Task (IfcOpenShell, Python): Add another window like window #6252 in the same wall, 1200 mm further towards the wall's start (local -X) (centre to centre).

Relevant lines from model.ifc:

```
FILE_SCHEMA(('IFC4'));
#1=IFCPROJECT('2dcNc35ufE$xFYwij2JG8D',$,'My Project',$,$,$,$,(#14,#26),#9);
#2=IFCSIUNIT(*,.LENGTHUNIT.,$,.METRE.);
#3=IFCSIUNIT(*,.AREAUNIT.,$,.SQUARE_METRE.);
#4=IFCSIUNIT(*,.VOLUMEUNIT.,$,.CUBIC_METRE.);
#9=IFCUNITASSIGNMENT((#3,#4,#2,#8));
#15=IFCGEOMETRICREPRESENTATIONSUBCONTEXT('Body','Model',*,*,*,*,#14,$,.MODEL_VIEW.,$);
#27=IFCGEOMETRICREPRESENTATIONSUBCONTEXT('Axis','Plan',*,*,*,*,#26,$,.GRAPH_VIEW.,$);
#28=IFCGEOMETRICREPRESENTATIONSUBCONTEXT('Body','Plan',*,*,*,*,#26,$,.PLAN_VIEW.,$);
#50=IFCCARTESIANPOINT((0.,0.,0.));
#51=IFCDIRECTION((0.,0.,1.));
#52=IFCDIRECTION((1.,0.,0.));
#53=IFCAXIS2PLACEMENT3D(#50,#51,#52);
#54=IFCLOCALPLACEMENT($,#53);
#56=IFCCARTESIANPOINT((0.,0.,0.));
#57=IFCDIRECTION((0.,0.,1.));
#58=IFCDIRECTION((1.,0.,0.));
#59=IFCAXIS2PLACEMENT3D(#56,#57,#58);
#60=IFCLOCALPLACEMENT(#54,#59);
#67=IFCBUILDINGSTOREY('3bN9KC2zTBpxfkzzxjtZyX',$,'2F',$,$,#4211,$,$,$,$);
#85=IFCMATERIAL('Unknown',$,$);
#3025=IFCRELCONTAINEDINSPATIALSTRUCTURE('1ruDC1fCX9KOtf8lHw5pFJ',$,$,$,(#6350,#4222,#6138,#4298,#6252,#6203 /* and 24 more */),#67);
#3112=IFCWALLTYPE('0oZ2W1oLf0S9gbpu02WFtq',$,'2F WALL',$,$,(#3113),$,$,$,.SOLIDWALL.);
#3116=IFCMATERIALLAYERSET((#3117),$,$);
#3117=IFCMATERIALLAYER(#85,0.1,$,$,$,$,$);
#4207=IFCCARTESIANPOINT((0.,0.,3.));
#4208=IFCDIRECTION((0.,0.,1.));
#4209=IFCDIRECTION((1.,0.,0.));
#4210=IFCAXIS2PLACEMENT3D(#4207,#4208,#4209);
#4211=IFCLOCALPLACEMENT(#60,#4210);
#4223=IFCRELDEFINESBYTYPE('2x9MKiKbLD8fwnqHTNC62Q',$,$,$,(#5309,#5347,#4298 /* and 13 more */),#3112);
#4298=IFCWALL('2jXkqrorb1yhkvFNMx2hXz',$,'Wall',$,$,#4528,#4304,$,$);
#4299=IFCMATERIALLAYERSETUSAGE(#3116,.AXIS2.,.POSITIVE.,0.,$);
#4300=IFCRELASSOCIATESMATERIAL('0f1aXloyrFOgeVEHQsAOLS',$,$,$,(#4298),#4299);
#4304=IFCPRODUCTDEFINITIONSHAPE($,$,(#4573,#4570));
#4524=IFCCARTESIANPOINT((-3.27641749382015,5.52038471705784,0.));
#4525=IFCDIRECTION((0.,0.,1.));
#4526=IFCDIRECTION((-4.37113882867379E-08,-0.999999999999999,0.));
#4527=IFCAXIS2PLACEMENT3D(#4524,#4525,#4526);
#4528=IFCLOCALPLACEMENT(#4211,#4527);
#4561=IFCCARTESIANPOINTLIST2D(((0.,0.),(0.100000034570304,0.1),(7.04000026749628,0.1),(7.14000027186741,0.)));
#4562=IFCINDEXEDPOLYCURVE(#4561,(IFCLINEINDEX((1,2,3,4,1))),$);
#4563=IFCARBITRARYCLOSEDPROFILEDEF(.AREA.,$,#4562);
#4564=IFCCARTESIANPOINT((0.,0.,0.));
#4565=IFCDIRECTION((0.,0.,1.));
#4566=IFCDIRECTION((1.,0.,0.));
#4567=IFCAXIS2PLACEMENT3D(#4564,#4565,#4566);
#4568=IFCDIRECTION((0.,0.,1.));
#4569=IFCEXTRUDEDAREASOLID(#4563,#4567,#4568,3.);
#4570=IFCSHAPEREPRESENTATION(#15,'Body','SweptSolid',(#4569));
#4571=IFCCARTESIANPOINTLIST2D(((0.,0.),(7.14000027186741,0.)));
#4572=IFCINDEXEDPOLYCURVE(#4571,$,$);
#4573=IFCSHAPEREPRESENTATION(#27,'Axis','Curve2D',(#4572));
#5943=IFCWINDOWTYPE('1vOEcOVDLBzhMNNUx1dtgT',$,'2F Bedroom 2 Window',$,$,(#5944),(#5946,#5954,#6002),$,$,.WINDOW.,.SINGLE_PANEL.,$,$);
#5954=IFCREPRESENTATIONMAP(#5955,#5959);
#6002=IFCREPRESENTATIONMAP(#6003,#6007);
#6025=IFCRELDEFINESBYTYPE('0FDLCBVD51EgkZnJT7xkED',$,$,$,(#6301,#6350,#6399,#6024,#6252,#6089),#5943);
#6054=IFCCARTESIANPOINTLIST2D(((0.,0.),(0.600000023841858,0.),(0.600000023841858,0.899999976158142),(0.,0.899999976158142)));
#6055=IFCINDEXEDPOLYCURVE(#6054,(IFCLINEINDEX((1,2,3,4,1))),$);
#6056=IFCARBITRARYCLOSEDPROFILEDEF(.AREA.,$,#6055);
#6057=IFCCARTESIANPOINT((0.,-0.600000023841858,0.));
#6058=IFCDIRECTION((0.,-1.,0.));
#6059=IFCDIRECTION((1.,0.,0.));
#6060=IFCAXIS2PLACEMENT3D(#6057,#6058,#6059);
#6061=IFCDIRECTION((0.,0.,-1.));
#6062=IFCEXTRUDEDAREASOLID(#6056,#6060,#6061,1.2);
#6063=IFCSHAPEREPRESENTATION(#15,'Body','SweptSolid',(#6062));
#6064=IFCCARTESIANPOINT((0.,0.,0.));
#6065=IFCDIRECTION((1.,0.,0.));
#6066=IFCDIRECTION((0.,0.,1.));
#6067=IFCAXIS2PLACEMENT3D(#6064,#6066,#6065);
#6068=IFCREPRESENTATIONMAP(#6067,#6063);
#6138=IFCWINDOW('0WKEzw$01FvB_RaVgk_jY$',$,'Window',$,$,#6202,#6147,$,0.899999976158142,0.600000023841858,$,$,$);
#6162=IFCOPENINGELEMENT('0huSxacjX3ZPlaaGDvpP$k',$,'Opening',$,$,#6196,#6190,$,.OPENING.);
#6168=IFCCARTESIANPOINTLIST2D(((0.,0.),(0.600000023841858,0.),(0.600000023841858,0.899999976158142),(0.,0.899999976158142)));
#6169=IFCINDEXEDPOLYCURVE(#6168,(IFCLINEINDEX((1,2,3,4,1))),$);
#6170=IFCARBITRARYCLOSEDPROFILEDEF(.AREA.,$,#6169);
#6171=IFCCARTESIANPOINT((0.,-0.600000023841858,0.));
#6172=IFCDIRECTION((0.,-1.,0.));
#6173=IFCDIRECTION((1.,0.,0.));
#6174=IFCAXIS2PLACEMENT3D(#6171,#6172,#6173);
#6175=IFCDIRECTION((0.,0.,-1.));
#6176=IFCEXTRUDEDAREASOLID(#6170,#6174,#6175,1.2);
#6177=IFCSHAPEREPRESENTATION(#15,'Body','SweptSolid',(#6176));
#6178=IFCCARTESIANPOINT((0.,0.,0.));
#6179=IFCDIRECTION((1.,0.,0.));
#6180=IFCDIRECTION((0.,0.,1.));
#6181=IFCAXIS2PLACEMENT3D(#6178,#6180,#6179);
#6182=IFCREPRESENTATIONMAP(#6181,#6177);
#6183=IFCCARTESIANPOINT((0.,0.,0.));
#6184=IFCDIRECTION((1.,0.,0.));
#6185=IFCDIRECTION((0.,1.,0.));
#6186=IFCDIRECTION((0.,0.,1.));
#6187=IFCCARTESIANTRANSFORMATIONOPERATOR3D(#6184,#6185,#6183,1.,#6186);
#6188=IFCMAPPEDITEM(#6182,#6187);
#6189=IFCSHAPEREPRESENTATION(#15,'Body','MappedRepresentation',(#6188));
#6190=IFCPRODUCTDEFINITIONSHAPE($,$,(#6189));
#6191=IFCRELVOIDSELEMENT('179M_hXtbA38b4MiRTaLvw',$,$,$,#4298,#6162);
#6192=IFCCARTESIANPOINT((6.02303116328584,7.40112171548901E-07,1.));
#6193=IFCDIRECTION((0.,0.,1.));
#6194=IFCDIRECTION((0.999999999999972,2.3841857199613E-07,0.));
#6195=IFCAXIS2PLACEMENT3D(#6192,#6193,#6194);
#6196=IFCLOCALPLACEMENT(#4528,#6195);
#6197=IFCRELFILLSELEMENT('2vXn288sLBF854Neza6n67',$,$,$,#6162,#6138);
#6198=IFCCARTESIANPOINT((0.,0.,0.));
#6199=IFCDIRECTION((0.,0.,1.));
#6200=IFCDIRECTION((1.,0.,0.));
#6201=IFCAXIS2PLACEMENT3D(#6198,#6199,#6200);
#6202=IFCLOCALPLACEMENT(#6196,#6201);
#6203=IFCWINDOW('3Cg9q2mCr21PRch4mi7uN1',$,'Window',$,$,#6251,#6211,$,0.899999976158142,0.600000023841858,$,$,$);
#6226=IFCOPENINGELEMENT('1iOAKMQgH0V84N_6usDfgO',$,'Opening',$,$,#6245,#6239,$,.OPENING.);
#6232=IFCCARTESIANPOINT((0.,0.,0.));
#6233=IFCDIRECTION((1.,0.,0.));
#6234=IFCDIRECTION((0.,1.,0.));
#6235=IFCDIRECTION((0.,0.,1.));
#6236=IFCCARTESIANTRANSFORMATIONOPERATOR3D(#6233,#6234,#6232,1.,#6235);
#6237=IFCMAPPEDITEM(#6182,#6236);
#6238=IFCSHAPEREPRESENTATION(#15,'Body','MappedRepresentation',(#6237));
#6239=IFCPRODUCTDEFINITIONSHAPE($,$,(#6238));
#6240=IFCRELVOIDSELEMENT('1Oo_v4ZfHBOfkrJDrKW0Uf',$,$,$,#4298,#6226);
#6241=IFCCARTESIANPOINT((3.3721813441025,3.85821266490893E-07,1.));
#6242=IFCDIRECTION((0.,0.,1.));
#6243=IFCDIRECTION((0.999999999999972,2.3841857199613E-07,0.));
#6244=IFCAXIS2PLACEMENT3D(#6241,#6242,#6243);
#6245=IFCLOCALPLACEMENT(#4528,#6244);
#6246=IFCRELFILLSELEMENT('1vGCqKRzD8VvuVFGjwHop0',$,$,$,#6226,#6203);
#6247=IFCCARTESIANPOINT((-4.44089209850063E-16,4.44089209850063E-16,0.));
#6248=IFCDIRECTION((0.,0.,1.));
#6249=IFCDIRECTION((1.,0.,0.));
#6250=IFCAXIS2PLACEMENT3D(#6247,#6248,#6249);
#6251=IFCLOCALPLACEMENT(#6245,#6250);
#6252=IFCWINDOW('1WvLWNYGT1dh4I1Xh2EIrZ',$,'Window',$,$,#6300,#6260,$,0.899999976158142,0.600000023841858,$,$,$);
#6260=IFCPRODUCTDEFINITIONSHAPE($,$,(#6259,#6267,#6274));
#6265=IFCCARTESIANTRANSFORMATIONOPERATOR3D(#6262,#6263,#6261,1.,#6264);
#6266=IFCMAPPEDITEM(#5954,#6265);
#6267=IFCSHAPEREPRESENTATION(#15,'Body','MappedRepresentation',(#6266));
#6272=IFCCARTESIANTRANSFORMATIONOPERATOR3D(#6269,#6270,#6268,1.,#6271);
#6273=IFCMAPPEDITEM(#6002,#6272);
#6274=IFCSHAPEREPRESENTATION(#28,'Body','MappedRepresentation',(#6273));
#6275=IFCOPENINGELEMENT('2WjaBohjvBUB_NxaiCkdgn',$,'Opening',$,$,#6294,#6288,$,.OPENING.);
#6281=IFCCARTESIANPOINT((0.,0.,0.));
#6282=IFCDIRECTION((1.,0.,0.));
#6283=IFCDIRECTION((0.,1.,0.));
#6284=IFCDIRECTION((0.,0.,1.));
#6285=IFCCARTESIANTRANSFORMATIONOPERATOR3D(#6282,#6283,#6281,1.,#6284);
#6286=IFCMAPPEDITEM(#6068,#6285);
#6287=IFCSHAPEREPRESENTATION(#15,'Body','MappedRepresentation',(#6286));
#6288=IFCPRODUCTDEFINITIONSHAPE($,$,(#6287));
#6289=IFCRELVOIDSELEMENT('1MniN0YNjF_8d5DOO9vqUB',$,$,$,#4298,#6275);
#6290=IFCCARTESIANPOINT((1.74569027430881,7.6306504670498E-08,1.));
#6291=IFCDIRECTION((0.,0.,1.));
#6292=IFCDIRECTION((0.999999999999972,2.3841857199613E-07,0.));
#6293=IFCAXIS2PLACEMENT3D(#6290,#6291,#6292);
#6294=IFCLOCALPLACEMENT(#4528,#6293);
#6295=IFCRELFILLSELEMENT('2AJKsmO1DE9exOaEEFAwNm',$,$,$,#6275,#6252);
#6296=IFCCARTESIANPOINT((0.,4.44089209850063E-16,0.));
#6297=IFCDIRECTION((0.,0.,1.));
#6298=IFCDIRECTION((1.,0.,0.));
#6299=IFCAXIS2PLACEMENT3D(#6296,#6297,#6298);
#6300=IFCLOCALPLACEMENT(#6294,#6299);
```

```python
import ifcopenshell
import ifcopenshell.api.feature
import ifcopenshell.api.geometry
import ifcopenshell.api.root
import ifcopenshell.geom
import ifcopenshell.util.element
import ifcopenshell.util.placement
import ifcopenshell.util.shape
import ifcopenshell.util.unit

model = ifcopenshell.open("model.ifc")
unit_scale = ifcopenshell.util.unit.calculate_unit_scale(model)
settings = ifcopenshell.geom.settings()


def volume(element):
    """Net volume in cubic metres, openings subtracted."""
    shape = ifcopenshell.geom.create_shape(settings, element)
    return ifcopenshell.util.shape.get_volume(shape.geometry)


window = model.by_id(6252)
opening = window.FillsVoids[0].RelatingOpeningElement
wall = opening.VoidsElements[0].RelatingBuildingElement
before = volume(wall)
shift = ifcopenshell.util.placement.get_local_placement(wall.ObjectPlacement)[:3, 0] * -1.2 / unit_scale

# copy_class copies the void relationship, type, container and properties, but no geometry.
new_opening = ifcopenshell.api.root.copy_class(model, product=opening)
new_opening.Representation = ifcopenshell.util.element.copy_deep(
    model, opening.Representation, exclude=["IfcGeometricRepresentationContext", "IfcRepresentationMap"]
)
new_window = ifcopenshell.api.root.copy_class(model, product=window)
new_window.Representation = ifcopenshell.util.element.copy_deep(
    model, window.Representation, exclude=["IfcGeometricRepresentationContext", "IfcRepresentationMap"]
)
ifcopenshell.api.feature.add_filling(model, opening=new_opening, element=new_window)

for old, new in ((opening, new_opening), (window, new_window)):
    matrix = ifcopenshell.util.placement.get_local_placement(old.ObjectPlacement)
    matrix[:3, 3] += shift
    ifcopenshell.api.geometry.edit_object_placement(model, product=new, matrix=matrix, is_si=False)

after = volume(wall)

print(f"wall volume {before:.3f} -> {after:.3f} m3")

model.write("model_v2.ifc")
```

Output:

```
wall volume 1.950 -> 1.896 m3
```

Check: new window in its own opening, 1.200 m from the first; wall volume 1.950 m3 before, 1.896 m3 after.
